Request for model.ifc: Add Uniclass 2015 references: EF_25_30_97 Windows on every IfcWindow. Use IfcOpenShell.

First a look at what the model holds.

```python
import ifcopenshell

model = ifcopenshell.open("model.ifc")
print(model.schema)
print("classifications:", [c.Name for c in model.by_type("IfcClassification")])
for ifc_class in ("IfcDoor", "IfcRoof", "IfcStair", "IfcWall", "IfcWindow"):
    print(ifc_class, len(model.by_type(ifc_class)))
```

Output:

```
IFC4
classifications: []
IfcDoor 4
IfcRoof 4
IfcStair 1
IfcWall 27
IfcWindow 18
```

```python
import ifcopenshell
import ifcopenshell.api.classification

model = ifcopenshell.open("model.ifc")

system = ifcopenshell.api.classification.add_classification(model, classification="Uniclass 2015")

codes = {
    "IfcWindow": ("EF_25_30_97", "Windows"),
}
for ifc_class, (code, name) in codes.items():
    products = model.by_type(ifc_class)
    ifcopenshell.api.classification.add_reference(
        model, products=products, classification=system, identification=code, name=name
    )
    print(code, len(products))

model.write("model_v2.ifc")
```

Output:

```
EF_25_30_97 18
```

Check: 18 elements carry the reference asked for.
